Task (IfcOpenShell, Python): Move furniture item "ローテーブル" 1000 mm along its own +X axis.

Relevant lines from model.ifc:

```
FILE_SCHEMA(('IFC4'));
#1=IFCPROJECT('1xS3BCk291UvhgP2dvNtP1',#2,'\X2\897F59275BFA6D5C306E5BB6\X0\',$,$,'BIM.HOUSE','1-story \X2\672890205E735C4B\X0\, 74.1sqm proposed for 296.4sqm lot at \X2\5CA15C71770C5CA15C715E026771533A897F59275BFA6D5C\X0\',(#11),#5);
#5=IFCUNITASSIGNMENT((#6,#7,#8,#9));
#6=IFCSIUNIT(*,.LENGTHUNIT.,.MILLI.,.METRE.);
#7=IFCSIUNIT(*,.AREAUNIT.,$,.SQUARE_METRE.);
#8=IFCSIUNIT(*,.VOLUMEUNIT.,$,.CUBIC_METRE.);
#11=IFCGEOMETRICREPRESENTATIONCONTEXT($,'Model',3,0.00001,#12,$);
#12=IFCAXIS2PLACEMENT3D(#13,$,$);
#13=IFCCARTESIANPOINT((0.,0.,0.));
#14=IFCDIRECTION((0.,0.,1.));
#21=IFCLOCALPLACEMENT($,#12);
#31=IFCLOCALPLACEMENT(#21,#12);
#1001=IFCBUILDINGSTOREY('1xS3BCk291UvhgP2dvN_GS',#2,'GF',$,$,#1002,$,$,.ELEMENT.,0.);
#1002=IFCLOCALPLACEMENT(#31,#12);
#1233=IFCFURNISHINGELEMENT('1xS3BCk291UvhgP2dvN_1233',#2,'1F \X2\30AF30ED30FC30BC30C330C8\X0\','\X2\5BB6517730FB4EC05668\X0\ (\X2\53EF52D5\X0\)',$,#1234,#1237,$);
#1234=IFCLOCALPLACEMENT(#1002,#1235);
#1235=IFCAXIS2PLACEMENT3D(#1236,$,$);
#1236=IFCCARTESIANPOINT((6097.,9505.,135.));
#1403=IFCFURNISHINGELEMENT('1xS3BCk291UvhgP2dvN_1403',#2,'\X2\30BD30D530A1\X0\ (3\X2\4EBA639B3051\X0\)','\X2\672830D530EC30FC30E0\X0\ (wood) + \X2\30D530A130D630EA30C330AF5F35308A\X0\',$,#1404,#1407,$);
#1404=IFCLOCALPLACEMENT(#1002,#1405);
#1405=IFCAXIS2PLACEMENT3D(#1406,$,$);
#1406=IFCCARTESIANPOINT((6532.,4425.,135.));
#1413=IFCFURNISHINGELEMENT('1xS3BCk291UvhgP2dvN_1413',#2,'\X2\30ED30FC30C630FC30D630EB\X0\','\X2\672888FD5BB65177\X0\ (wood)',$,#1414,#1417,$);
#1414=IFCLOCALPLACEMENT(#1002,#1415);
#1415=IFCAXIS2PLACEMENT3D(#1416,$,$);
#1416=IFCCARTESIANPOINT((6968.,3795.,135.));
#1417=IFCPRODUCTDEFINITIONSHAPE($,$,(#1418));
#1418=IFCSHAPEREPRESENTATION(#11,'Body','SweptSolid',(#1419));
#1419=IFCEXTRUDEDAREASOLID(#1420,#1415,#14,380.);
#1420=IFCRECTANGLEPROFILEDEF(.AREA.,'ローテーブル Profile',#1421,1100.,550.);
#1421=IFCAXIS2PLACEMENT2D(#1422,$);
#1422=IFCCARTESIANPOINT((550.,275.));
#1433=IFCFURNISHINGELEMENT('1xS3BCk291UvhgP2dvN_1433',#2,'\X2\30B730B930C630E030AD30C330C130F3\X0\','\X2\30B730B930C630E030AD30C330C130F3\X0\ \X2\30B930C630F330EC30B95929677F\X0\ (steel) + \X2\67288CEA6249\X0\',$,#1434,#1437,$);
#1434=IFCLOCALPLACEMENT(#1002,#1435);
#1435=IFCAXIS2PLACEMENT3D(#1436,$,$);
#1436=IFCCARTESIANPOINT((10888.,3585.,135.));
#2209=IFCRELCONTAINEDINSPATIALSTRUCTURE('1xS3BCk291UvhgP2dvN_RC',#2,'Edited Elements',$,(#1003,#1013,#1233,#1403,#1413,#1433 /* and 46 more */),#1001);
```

```python
import ifcopenshell
import ifcopenshell.api.geometry
import ifcopenshell.util.placement

model = ifcopenshell.open("model.ifc")

item = model.by_id(1413)
matrix = ifcopenshell.util.placement.get_local_placement(item.ObjectPlacement)
matrix[:3, 3] += matrix[:3, 0] * 1000.0
ifcopenshell.api.geometry.edit_object_placement(model, product=item, matrix=matrix, is_si=False)

print(ifcopenshell.util.placement.get_local_placement(item.ObjectPlacement).round(3) + 0.0)

model.write("model-out.ifc")
```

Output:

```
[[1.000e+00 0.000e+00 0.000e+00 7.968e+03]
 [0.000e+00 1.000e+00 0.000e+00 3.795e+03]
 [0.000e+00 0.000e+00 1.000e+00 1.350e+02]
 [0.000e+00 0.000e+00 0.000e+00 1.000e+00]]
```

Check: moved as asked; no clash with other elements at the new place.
